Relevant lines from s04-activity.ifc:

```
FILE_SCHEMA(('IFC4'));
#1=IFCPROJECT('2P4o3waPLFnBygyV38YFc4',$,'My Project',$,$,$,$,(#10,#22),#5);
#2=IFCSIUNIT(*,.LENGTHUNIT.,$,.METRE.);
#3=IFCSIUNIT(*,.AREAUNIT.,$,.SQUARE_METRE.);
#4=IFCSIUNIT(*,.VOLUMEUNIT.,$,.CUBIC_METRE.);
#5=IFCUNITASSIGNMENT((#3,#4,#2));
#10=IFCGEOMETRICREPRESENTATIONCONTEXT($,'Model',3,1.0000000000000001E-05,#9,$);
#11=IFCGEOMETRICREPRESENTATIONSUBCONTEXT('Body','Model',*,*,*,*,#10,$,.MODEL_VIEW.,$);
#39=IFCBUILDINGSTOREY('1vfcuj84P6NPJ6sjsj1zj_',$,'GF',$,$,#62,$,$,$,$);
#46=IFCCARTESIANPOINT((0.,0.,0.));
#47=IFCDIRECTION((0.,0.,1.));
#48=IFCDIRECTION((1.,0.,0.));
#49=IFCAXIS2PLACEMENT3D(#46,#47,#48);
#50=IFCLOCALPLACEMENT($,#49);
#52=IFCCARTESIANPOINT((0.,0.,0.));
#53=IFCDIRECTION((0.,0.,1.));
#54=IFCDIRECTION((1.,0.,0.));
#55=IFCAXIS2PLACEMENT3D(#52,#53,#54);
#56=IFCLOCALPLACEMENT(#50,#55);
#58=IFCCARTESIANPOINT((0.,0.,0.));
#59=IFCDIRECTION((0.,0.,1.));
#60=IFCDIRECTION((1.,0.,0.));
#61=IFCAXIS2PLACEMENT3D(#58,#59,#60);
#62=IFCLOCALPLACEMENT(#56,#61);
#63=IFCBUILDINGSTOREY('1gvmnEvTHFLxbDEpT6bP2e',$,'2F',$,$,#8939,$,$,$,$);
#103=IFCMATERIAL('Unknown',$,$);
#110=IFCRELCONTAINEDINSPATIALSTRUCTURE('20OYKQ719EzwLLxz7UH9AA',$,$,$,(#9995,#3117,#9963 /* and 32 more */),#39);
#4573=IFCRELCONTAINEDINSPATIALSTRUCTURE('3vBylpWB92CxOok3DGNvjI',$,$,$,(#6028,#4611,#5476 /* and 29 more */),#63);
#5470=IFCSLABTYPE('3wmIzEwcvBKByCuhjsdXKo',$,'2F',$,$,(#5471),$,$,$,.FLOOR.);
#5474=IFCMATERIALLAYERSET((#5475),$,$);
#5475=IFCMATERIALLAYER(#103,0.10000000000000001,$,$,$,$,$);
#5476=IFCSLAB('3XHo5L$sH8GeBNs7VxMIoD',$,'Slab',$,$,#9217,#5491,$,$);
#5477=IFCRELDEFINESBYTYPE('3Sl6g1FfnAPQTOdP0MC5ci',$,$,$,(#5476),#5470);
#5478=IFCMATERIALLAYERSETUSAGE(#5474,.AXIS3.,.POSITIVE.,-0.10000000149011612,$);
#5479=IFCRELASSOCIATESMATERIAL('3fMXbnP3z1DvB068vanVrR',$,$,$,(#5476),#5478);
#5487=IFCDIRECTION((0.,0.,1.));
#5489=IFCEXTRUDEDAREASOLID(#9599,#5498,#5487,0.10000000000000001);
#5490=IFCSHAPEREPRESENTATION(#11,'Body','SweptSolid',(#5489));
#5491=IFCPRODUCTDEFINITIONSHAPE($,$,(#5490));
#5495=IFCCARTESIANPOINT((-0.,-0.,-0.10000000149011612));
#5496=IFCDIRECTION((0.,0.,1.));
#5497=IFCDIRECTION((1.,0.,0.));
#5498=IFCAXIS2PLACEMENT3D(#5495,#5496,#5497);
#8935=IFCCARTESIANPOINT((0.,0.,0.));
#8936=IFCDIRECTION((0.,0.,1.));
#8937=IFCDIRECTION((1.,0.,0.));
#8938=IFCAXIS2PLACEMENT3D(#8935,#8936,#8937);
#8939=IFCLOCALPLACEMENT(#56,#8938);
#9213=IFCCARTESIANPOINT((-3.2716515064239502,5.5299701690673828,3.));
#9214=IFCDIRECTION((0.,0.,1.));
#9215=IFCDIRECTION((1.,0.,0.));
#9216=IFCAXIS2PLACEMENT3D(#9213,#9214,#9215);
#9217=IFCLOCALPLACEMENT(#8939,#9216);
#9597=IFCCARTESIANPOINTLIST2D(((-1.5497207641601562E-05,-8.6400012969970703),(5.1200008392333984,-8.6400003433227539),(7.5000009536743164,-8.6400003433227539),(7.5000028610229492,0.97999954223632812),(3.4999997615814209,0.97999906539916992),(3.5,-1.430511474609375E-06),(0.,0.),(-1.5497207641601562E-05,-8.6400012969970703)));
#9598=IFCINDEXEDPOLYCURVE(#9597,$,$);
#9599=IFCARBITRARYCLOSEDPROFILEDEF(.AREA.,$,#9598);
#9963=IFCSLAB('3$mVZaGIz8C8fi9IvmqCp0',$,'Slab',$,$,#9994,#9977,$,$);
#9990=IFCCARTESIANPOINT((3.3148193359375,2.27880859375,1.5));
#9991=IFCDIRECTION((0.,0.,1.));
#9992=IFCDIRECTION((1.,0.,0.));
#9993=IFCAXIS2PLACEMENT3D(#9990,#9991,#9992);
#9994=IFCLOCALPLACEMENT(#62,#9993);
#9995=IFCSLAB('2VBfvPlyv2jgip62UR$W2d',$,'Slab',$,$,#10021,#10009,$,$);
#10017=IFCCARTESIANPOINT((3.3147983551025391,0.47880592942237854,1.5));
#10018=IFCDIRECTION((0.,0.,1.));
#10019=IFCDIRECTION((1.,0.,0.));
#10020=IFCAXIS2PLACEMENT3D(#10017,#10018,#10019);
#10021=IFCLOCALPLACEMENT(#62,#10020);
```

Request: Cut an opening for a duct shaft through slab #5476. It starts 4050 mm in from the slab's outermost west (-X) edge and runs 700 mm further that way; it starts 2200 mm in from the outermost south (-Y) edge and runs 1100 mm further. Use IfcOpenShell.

```python
import numpy as np
import ifcopenshell
import ifcopenshell.api.feature
import ifcopenshell.api.geometry
import ifcopenshell.api.root
import ifcopenshell.geom
import ifcopenshell.util.placement
import ifcopenshell.util.representation
import ifcopenshell.util.shape
import ifcopenshell.util.unit

model = ifcopenshell.open("s04-activity.ifc")
unit_scale = ifcopenshell.util.unit.calculate_unit_scale(model)
settings = ifcopenshell.geom.settings()


def volume(element):
    """Net volume in cubic metres, openings subtracted."""
    shape = ifcopenshell.geom.create_shape(settings, element)
    return ifcopenshell.util.shape.get_volume(shape.geometry)


slab = model.by_guid("3XHo5L$sH8GeBNs7VxMIoD")
before = volume(slab)

# Extent in the slab's own axes, in metres. The edges named are its -X and -Y sides.
slab_shape = ifcopenshell.geom.create_shape(settings, slab)
vertices = ifcopenshell.util.shape.get_vertices(slab_shape.geometry)
x_min, y_min, bottom = vertices.min(axis=0)
top = vertices[:, 2].max()

opening = ifcopenshell.api.root.create_entity(model, ifc_class="IfcOpeningElement", name="Duct shaft opening", predefined_type="OPENING")
context = ifcopenshell.util.representation.get_context(model, "Model", "Body", "MODEL_VIEW")
width, depth = 0.7, 1.1
outline = [(0.0, 0.0), (width, 0.0), (width, depth), (0.0, depth), (0.0, 0.0)]
# Overshoot both faces by 50 mm so the cut is clean.
shape = ifcopenshell.api.geometry.add_slab_representation(
    model, context=context, depth=top - bottom + 0.1, polyline=outline
)
ifcopenshell.api.geometry.assign_representation(model, product=opening, representation=shape)

matrix = ifcopenshell.util.placement.get_local_placement(slab.ObjectPlacement)
matrix[:, 3] = matrix @ np.append(np.array([x_min + 4.05, y_min + 2.2, bottom - 0.05]) / unit_scale, 1.0)
ifcopenshell.api.geometry.edit_object_placement(model, product=opening, matrix=matrix, is_si=False)
ifcopenshell.api.feature.add_feature(model, feature=opening, element=slab)

after = volume(slab)

print(f"slab volume {before:.3f} -> {after:.3f} m3")

model.write("s04-activity_updated.ifc")
```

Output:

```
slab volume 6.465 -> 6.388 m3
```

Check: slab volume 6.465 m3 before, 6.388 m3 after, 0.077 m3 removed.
